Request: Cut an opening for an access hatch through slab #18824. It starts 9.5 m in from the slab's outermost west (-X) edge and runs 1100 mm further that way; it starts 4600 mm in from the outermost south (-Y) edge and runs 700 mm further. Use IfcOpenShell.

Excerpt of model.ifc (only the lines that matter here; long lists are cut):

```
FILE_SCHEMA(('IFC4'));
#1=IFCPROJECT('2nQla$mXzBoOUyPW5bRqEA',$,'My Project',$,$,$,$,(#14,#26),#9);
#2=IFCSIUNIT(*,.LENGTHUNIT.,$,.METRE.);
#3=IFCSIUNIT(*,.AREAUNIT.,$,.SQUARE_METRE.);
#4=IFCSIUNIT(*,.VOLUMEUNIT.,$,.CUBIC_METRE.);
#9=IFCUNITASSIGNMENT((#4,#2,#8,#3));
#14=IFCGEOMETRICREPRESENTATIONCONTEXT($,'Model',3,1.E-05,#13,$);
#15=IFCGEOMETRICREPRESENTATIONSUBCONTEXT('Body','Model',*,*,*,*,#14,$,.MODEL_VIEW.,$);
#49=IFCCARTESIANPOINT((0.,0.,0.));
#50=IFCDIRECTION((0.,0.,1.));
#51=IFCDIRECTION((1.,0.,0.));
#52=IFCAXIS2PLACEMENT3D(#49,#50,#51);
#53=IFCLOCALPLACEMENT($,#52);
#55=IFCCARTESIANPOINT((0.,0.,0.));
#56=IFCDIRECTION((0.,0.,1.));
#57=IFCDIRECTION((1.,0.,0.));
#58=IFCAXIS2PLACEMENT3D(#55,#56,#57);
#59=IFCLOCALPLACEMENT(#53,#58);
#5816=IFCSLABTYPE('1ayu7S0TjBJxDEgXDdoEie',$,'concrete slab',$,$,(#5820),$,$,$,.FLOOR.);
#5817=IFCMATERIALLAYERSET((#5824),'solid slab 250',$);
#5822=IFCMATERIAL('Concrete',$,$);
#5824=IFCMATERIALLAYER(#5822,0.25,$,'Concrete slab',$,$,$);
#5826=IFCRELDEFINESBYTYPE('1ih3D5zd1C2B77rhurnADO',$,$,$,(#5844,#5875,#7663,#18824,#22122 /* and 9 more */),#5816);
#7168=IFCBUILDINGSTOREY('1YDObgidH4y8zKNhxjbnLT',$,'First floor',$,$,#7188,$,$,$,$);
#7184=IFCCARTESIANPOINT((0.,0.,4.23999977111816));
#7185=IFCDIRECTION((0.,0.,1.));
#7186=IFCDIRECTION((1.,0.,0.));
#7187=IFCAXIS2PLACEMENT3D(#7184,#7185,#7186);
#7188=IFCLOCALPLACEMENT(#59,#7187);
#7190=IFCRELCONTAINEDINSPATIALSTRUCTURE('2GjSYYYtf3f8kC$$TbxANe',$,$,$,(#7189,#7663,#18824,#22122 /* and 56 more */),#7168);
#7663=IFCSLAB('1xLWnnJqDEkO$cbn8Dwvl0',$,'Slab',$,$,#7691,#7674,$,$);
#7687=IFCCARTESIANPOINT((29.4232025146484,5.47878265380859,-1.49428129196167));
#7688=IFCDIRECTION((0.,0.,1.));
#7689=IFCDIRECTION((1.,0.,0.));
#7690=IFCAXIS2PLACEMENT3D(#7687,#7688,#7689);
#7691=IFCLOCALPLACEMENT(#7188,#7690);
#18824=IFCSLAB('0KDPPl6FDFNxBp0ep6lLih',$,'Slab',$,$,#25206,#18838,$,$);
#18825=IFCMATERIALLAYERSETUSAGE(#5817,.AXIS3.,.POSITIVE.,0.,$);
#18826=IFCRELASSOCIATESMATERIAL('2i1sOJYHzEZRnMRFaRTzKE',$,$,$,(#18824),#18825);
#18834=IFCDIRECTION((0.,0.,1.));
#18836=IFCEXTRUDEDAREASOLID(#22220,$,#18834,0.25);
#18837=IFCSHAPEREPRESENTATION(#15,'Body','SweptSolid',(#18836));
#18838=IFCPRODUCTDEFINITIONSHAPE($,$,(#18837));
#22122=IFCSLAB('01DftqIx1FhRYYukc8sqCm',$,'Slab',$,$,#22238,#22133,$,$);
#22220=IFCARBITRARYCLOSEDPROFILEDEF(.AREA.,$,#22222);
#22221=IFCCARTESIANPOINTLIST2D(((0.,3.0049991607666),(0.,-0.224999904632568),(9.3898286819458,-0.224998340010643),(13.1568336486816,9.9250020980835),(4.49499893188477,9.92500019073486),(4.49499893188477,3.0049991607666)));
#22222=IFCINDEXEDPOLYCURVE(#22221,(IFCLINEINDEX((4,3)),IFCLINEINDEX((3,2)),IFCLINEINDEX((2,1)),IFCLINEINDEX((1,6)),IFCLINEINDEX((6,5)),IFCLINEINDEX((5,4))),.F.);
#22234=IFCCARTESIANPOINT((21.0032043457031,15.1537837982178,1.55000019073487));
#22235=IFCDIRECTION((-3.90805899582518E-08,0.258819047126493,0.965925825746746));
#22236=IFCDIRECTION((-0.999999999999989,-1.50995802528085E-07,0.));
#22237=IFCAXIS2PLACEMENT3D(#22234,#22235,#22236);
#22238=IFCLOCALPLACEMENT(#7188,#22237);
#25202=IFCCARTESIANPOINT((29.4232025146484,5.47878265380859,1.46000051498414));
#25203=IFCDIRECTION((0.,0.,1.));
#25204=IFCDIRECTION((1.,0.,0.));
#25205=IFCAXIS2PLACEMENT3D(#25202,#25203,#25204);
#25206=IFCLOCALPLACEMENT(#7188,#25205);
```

```python
import numpy as np
import ifcopenshell
import ifcopenshell.api.feature
import ifcopenshell.api.geometry
import ifcopenshell.api.root
import ifcopenshell.geom
import ifcopenshell.util.placement
import ifcopenshell.util.representation
import ifcopenshell.util.shape
import ifcopenshell.util.unit

model = ifcopenshell.open("model.ifc")
unit_scale = ifcopenshell.util.unit.calculate_unit_scale(model)
settings = ifcopenshell.geom.settings()


def volume(element):
    """Net volume in cubic metres, openings subtracted."""
    shape = ifcopenshell.geom.create_shape(settings, element)
    return ifcopenshell.util.shape.get_volume(shape.geometry)


slab = model.by_guid("0KDPPl6FDFNxBp0ep6lLih")
before = volume(slab)

# Extent in the slab's own axes, in metres. The edges named are its -X and -Y sides.
slab_shape = ifcopenshell.geom.create_shape(settings, slab)
vertices = ifcopenshell.util.shape.get_vertices(slab_shape.geometry)
x_min, y_min, bottom = vertices.min(axis=0)
top = vertices[:, 2].max()

opening = ifcopenshell.api.root.create_entity(model, ifc_class="IfcOpeningElement", name="Access hatch opening", predefined_type="OPENING")
context = ifcopenshell.util.representation.get_context(model, "Model", "Body", "MODEL_VIEW")
width, depth = 1.1, 0.7
outline = [(0.0, 0.0), (width, 0.0), (width, depth), (0.0, depth), (0.0, 0.0)]
# Overshoot both faces by 50 mm so the cut is clean.
shape = ifcopenshell.api.geometry.add_slab_representation(
    model, context=context, depth=top - bottom + 0.1, polyline=outline
)
ifcopenshell.api.geometry.assign_representation(model, product=opening, representation=shape)

matrix = ifcopenshell.util.placement.get_local_placement(slab.ObjectPlacement)
matrix[:, 3] = matrix @ np.append(np.array([x_min + 9.5, y_min + 4.6, bottom - 0.05]) / unit_scale, 1.0)
ifcopenshell.api.geometry.edit_object_placement(model, product=opening, matrix=matrix, is_si=False)
ifcopenshell.api.feature.add_feature(model, feature=opening, element=slab)

after = volume(slab)

print(f"slab volume {before:.3f} -> {after:.3f} m3")

model.write("model-out.ifc")
```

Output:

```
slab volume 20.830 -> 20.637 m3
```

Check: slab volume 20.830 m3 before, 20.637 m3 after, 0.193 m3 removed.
